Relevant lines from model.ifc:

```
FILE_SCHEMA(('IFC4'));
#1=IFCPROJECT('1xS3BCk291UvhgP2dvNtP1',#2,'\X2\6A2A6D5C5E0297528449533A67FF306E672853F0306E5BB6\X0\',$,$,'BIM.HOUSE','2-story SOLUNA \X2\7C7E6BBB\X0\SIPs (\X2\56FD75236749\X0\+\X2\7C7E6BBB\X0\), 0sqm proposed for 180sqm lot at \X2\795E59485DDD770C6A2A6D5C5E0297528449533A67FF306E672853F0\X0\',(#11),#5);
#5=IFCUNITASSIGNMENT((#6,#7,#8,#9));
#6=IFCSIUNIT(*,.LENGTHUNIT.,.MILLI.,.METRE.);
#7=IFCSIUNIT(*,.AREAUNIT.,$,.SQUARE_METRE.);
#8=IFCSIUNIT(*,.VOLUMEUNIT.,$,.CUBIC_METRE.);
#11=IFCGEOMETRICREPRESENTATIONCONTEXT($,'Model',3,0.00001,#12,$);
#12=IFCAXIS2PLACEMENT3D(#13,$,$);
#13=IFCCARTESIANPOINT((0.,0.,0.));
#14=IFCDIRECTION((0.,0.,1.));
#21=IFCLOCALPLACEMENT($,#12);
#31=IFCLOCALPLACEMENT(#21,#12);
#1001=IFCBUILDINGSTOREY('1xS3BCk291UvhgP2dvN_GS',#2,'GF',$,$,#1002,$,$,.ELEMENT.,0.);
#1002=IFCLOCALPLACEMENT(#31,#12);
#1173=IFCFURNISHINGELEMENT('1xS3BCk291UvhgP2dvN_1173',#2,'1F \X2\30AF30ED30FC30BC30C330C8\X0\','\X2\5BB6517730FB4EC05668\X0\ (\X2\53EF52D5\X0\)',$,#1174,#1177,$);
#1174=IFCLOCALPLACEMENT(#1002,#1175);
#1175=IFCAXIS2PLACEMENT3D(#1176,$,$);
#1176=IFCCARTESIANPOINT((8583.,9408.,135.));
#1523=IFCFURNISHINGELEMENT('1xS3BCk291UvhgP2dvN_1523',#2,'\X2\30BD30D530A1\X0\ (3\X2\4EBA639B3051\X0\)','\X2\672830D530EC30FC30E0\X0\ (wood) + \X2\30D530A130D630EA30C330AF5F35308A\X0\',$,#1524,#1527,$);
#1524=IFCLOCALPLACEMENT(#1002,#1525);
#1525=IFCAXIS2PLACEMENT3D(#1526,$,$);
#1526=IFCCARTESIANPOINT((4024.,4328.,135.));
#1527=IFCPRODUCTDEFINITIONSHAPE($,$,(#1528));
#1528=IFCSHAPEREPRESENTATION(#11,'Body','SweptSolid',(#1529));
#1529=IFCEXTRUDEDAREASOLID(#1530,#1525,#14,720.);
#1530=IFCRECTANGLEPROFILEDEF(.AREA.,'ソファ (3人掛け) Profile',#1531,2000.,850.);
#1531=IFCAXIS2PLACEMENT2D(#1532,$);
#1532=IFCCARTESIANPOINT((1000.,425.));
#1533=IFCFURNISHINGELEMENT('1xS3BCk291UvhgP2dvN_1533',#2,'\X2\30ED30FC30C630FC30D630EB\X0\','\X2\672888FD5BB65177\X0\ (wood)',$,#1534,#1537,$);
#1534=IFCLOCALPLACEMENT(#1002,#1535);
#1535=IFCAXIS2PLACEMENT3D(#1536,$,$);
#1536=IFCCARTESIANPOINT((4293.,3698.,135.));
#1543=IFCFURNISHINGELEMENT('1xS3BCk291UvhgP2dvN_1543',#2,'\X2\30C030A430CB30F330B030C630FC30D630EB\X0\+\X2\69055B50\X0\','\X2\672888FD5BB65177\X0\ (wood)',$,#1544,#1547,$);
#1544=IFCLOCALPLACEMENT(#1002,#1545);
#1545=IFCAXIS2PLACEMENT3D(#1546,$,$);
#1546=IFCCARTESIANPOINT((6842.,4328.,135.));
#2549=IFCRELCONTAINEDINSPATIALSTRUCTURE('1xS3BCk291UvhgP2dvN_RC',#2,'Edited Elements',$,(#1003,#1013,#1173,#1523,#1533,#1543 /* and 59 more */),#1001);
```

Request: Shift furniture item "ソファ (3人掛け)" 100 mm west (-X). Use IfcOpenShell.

```python
import ifcopenshell
import ifcopenshell.api.geometry
import ifcopenshell.util.placement
import ifcopenshell.util.unit

model = ifcopenshell.open("model.ifc")
unit_scale = ifcopenshell.util.unit.calculate_unit_scale(model)

item = model.by_id(1523)
matrix = ifcopenshell.util.placement.get_local_placement(item.ObjectPlacement)
matrix[0, 3] -= 0.1 / unit_scale
ifcopenshell.api.geometry.edit_object_placement(model, product=item, matrix=matrix, is_si=False)

print(ifcopenshell.util.placement.get_local_placement(item.ObjectPlacement).round(3) + 0.0)

model.write("model_rev.ifc")
```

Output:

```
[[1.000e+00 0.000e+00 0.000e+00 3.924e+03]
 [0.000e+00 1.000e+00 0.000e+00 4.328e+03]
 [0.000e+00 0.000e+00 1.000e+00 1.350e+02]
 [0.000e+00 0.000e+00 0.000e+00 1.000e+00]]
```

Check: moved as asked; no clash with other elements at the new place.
